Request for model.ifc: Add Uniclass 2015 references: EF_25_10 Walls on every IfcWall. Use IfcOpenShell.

First a look at what the model holds.

```python
import ifcopenshell

model = ifcopenshell.open("model.ifc")
print(model.schema)
print("classifications:", [c.Name for c in model.by_type("IfcClassification")])
for ifc_class in ("IfcDoor", "IfcRoof", "IfcStair", "IfcWall", "IfcWindow"):
    print(ifc_class, len(model.by_type(ifc_class)))
```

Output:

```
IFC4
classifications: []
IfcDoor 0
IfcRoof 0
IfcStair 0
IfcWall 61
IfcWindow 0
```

```python
import ifcopenshell
import ifcopenshell.api.classification

model = ifcopenshell.open("model.ifc")

system = ifcopenshell.api.classification.add_classification(model, classification="Uniclass 2015")

codes = {
    "IfcWall": ("EF_25_10", "Walls"),
}
for ifc_class, (code, name) in codes.items():
    products = model.by_type(ifc_class)
    ifcopenshell.api.classification.add_reference(
        model, products=products, classification=system, identification=code, name=name
    )
    print(code, len(products))

model.write("model_v2.ifc")
```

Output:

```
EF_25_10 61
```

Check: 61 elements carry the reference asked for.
